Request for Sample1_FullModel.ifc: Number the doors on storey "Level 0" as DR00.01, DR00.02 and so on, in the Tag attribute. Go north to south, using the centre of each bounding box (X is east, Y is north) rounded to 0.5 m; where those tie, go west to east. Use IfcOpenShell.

First a look at what the model holds.

```python
import ifcopenshell
import ifcopenshell.util.element
import ifcopenshell.util.placement

model = ifcopenshell.open("Sample1_FullModel.ifc")
print(model.schema)
storey = next(s for s in model.by_type("IfcBuildingStorey") if s.Name == "Level 0")
doors = [e for e in ifcopenshell.util.element.get_decomposition(storey) if e.is_a("IfcDoor")]
for e in sorted(doors, key=lambda e: e.id()):
    origin = ifcopenshell.util.placement.get_local_placement(e.ObjectPlacement)[:3, 3]
    print(e.id(), e.Tag, e.Name, origin.round(2) + 0.0, sep=" | ")
```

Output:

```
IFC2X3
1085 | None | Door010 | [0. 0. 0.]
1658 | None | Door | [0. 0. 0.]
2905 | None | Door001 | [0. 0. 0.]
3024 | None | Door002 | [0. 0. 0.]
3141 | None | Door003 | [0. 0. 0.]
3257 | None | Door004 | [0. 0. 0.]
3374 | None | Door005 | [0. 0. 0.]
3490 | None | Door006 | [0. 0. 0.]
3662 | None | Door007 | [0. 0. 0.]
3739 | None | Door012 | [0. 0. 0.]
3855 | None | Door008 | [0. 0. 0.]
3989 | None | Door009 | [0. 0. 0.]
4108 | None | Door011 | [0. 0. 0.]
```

```python
import ifcopenshell
import ifcopenshell.geom
import ifcopenshell.util.element
import ifcopenshell.util.shape

model = ifcopenshell.open("Sample1_FullModel.ifc")
settings = ifcopenshell.geom.settings()
settings.set("use-world-coords", True)


def centre(element):
    shape = ifcopenshell.geom.create_shape(settings, element)
    return ifcopenshell.util.shape.get_bbox_centroid(shape.geometry)


storey = next(s for s in model.by_type("IfcBuildingStorey") if s.Name == "Level 0")
doors = [e for e in ifcopenshell.util.element.get_decomposition(storey) if e.is_a("IfcDoor")]

# Insertion points can sit at a corner or the storey origin, so sort by the geometry (in metres).
centres = {e: centre(e) for e in doors}
doors.sort(key=lambda e: (-round(centres[e][1] / 0.5), centres[e][0]))

for i, e in enumerate(doors, start=1):
    number = f"DR00.{i:02d}"
    e.Tag = number
    print(e.id(), number)

model.write("Sample1_FullModel_edited.ifc")
```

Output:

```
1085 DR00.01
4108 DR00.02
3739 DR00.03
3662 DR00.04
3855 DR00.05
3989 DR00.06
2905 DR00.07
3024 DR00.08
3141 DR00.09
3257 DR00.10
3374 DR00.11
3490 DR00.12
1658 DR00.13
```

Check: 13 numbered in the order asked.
